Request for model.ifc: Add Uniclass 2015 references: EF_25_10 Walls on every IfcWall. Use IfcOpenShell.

First a look at what the model holds.

```python
import ifcopenshell

model = ifcopenshell.open("model.ifc")
print(model.schema)
print("classifications:", [c.Name for c in model.by_type("IfcClassification")])
for ifc_class in ("IfcDoor", "IfcRoof", "IfcStair", "IfcWall", "IfcWindow"):
    print(ifc_class, len(model.by_type(ifc_class)))
```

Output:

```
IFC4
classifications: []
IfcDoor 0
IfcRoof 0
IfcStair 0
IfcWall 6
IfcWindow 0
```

```python
import ifcopenshell
import ifcopenshell.api.classification

model = ifcopenshell.open("model.ifc")

system = ifcopenshell.api.classification.add_classification(model, classification="Uniclass 2015")

codes = {
    "IfcWall": ("EF_25_10", "Walls"),
}
for ifc_class, (code, name) in codes.items():
    products = model.by_type(ifc_class)
    ifcopenshell.api.classification.add_reference(
        model, products=products, classification=system, identification=code, name=name
    )
    print(code, len(products))

model.write("model_updated.ifc")
```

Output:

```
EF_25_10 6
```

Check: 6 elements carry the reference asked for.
